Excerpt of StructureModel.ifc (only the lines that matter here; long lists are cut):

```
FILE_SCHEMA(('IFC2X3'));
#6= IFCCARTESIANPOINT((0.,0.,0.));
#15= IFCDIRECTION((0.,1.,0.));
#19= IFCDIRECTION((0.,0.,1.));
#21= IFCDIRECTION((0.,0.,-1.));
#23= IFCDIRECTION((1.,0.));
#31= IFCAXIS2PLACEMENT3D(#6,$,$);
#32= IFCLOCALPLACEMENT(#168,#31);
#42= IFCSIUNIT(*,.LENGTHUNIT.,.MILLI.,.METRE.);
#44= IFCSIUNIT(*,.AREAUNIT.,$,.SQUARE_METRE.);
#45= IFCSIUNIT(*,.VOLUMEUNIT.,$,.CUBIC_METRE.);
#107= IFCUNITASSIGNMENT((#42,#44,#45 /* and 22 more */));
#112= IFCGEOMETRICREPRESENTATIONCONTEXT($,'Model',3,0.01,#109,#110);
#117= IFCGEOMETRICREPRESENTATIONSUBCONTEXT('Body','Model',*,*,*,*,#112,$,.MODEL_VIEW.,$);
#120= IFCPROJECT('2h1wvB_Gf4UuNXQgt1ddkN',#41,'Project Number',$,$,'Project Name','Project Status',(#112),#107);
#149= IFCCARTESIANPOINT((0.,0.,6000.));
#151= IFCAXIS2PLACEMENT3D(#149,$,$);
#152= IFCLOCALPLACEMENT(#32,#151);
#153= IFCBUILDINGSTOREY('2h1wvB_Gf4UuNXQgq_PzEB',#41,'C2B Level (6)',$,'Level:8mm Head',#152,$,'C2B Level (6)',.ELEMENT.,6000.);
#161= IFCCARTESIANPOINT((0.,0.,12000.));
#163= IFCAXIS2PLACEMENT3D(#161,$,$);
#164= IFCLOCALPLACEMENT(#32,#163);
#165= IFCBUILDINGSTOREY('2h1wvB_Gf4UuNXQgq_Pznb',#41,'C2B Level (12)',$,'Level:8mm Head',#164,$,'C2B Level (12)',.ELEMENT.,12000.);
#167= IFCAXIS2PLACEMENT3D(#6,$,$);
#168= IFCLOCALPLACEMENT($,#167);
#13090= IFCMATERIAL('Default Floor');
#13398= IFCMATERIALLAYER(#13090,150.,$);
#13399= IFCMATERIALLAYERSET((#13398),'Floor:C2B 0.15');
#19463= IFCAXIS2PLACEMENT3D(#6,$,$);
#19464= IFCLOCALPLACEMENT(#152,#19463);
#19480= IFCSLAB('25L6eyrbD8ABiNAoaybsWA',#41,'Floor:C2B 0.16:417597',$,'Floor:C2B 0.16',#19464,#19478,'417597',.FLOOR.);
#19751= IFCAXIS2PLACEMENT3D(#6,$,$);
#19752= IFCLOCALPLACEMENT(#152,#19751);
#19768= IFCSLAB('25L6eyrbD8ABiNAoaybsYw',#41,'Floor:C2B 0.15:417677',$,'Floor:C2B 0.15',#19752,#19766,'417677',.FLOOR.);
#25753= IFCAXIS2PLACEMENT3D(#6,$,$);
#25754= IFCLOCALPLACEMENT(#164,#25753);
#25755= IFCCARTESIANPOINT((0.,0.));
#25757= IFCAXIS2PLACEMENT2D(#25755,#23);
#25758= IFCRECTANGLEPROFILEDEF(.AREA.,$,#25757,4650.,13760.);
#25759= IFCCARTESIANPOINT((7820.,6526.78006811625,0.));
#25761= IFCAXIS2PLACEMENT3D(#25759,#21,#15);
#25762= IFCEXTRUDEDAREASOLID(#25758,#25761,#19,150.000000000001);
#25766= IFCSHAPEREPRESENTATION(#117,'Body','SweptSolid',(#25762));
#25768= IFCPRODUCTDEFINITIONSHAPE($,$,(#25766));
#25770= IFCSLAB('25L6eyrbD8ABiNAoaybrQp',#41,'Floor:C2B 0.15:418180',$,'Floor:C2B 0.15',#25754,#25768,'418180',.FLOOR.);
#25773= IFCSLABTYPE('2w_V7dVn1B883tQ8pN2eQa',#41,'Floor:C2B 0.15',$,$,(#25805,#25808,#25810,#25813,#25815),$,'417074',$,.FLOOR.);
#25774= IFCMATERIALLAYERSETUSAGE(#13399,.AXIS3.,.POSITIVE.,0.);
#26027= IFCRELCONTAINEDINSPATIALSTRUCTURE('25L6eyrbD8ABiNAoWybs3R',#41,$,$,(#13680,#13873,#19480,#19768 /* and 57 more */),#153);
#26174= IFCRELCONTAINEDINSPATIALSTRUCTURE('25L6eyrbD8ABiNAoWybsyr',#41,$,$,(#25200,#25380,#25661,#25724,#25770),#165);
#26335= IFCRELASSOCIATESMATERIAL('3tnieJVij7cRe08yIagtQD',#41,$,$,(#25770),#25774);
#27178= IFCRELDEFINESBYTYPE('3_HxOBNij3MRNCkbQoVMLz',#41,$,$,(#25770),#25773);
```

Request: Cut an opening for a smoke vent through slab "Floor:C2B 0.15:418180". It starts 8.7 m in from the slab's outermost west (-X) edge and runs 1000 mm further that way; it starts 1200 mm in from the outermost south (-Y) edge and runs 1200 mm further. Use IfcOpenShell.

```python
import numpy as np
import ifcopenshell
import ifcopenshell.api.feature
import ifcopenshell.api.geometry
import ifcopenshell.api.root
import ifcopenshell.geom
import ifcopenshell.util.placement
import ifcopenshell.util.representation
import ifcopenshell.util.shape
import ifcopenshell.util.unit

model = ifcopenshell.open("StructureModel.ifc")
unit_scale = ifcopenshell.util.unit.calculate_unit_scale(model)
settings = ifcopenshell.geom.settings()


def volume(element):
    """Net volume in cubic metres, openings subtracted."""
    shape = ifcopenshell.geom.create_shape(settings, element)
    return ifcopenshell.util.shape.get_volume(shape.geometry)


slab = model.by_guid("25L6eyrbD8ABiNAoaybrQp")
before = volume(slab)

# Extent in the slab's own axes, in metres. The edges named are its -X and -Y sides.
slab_shape = ifcopenshell.geom.create_shape(settings, slab)
vertices = ifcopenshell.util.shape.get_vertices(slab_shape.geometry)
x_min, y_min, bottom = vertices.min(axis=0)
top = vertices[:, 2].max()

opening = ifcopenshell.api.root.create_entity(model, ifc_class="IfcOpeningElement", name="Smoke vent opening")
context = ifcopenshell.util.representation.get_context(model, "Model", "Body", "MODEL_VIEW")
width, depth = 1, 1.2
outline = [(0.0, 0.0), (width, 0.0), (width, depth), (0.0, depth), (0.0, 0.0)]
# Overshoot both faces by 50 mm so the cut is clean.
shape = ifcopenshell.api.geometry.add_slab_representation(
    model, context=context, depth=top - bottom + 0.1, polyline=outline
)
ifcopenshell.api.geometry.assign_representation(model, product=opening, representation=shape)

matrix = ifcopenshell.util.placement.get_local_placement(slab.ObjectPlacement)
matrix[:, 3] = matrix @ np.append(np.array([x_min + 8.7, y_min + 1.2, bottom - 0.05]) / unit_scale, 1.0)
ifcopenshell.api.geometry.edit_object_placement(model, product=opening, matrix=matrix, is_si=False)
ifcopenshell.api.feature.add_feature(model, feature=opening, element=slab)

after = volume(slab)

print(f"slab volume {before:.3f} -> {after:.3f} m3")

model.write("StructureModel-out.ifc")
```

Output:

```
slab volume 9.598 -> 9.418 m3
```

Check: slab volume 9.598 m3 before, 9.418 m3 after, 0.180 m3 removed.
